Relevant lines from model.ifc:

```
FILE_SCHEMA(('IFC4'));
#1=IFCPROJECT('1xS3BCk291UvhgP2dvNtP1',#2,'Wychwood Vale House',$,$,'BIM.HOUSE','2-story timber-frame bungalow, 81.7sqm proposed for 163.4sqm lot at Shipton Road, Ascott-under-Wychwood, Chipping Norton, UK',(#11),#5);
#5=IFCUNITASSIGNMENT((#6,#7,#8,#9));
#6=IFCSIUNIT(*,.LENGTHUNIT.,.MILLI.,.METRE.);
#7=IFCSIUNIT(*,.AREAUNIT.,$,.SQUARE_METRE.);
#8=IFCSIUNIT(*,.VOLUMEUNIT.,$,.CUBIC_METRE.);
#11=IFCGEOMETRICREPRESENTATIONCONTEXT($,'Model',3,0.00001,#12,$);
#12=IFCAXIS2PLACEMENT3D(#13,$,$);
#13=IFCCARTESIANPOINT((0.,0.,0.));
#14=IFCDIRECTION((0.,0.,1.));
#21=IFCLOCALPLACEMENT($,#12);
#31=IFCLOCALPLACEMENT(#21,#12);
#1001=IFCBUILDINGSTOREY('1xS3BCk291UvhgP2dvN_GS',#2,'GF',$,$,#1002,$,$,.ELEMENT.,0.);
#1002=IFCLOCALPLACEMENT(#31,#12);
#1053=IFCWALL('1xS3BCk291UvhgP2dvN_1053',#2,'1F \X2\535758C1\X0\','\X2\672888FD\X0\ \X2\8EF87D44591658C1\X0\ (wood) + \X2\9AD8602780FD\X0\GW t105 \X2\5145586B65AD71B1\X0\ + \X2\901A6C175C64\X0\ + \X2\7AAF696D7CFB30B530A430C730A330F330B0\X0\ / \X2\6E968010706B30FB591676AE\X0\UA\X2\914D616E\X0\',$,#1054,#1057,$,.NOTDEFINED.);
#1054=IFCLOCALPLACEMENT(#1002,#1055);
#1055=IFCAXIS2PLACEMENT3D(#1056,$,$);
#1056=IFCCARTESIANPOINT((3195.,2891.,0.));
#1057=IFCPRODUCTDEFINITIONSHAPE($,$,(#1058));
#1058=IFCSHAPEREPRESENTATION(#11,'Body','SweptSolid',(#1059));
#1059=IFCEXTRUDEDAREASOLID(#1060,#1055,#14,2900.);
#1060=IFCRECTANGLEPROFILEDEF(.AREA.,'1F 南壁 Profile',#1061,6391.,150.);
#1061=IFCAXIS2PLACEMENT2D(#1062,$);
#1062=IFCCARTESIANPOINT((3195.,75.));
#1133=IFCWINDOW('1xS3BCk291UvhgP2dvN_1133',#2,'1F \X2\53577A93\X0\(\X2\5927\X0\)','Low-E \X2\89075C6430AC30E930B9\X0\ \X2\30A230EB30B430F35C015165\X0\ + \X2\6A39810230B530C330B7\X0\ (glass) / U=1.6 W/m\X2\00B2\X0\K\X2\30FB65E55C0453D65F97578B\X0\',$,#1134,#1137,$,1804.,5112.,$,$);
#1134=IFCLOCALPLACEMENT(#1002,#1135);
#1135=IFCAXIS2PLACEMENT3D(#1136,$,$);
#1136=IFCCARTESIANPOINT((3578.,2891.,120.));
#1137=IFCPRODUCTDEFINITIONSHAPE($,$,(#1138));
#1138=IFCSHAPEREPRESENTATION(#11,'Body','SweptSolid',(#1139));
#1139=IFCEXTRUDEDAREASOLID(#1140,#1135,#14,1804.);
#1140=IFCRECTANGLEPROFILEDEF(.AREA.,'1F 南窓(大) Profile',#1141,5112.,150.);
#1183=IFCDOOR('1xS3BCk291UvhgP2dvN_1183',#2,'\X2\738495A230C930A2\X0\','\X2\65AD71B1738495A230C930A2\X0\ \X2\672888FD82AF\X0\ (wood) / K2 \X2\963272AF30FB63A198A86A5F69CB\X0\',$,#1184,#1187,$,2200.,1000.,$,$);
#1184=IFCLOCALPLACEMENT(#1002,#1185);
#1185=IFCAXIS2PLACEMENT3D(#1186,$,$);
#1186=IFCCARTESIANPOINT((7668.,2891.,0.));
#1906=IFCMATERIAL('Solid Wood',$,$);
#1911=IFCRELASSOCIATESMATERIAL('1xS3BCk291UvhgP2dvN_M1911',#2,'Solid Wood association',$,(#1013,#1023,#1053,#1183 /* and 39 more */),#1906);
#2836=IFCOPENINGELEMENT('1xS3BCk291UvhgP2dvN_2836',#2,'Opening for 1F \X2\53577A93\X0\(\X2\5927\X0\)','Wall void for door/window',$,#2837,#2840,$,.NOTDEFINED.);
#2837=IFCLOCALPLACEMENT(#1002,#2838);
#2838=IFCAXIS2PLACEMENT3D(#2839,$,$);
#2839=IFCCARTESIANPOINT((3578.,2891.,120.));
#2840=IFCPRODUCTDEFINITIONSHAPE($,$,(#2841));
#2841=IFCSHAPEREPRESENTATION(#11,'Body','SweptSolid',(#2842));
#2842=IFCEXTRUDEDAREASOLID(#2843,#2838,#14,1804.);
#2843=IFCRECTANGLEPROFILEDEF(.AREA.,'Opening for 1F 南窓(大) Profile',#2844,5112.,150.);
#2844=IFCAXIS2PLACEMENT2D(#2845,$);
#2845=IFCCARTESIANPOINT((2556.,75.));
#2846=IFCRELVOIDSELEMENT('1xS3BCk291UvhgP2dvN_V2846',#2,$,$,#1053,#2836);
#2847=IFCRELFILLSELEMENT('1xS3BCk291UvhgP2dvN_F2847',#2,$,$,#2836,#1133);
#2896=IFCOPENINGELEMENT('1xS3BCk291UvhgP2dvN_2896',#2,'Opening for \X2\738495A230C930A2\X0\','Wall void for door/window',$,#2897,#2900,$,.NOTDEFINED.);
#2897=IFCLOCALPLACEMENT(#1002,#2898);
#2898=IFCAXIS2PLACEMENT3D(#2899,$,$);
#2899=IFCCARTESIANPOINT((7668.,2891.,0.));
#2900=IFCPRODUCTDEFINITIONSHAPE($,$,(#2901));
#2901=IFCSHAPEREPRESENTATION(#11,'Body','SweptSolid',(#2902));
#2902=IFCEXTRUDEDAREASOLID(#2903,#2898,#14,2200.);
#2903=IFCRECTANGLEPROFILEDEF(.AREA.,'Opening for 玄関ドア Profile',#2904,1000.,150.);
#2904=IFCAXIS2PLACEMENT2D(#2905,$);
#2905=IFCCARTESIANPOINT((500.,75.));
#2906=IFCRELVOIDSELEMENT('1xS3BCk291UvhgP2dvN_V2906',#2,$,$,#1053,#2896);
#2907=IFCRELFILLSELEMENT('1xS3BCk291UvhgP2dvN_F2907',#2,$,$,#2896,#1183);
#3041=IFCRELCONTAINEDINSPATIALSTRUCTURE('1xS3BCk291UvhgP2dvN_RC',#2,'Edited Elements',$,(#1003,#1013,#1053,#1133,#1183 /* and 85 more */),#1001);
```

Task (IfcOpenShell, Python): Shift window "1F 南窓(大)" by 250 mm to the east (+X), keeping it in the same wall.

```python
import ifcopenshell
import ifcopenshell.api.geometry
import ifcopenshell.util.placement

model = ifcopenshell.open("model.ifc")

window = model.by_guid("1xS3BCk291UvhgP2dvN_1133")
opening = window.FillsVoids[0].RelatingOpeningElement
wall = opening.VoidsElements[0].RelatingBuildingElement

wall_matrix = ifcopenshell.util.placement.get_local_placement(wall.ObjectPlacement)
shift = wall_matrix[:3, 0] * 250.0
before = ifcopenshell.util.placement.get_local_placement(window.ObjectPlacement)[:3, 3].copy()

# The window is not placed relative to its opening, so move both.
for product in (opening, window):
    matrix = ifcopenshell.util.placement.get_local_placement(product.ObjectPlacement)
    matrix[:3, 3] += shift
    ifcopenshell.api.geometry.edit_object_placement(model, product=product, matrix=matrix, is_si=False)

after = ifcopenshell.util.placement.get_local_placement(window.ObjectPlacement)[:3, 3]
print("window moved by", (after - before).round(3) + 0.0)

model.write("model_rev.ifc")
```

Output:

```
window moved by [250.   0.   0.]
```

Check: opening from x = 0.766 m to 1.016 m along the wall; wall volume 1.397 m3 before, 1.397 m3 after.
